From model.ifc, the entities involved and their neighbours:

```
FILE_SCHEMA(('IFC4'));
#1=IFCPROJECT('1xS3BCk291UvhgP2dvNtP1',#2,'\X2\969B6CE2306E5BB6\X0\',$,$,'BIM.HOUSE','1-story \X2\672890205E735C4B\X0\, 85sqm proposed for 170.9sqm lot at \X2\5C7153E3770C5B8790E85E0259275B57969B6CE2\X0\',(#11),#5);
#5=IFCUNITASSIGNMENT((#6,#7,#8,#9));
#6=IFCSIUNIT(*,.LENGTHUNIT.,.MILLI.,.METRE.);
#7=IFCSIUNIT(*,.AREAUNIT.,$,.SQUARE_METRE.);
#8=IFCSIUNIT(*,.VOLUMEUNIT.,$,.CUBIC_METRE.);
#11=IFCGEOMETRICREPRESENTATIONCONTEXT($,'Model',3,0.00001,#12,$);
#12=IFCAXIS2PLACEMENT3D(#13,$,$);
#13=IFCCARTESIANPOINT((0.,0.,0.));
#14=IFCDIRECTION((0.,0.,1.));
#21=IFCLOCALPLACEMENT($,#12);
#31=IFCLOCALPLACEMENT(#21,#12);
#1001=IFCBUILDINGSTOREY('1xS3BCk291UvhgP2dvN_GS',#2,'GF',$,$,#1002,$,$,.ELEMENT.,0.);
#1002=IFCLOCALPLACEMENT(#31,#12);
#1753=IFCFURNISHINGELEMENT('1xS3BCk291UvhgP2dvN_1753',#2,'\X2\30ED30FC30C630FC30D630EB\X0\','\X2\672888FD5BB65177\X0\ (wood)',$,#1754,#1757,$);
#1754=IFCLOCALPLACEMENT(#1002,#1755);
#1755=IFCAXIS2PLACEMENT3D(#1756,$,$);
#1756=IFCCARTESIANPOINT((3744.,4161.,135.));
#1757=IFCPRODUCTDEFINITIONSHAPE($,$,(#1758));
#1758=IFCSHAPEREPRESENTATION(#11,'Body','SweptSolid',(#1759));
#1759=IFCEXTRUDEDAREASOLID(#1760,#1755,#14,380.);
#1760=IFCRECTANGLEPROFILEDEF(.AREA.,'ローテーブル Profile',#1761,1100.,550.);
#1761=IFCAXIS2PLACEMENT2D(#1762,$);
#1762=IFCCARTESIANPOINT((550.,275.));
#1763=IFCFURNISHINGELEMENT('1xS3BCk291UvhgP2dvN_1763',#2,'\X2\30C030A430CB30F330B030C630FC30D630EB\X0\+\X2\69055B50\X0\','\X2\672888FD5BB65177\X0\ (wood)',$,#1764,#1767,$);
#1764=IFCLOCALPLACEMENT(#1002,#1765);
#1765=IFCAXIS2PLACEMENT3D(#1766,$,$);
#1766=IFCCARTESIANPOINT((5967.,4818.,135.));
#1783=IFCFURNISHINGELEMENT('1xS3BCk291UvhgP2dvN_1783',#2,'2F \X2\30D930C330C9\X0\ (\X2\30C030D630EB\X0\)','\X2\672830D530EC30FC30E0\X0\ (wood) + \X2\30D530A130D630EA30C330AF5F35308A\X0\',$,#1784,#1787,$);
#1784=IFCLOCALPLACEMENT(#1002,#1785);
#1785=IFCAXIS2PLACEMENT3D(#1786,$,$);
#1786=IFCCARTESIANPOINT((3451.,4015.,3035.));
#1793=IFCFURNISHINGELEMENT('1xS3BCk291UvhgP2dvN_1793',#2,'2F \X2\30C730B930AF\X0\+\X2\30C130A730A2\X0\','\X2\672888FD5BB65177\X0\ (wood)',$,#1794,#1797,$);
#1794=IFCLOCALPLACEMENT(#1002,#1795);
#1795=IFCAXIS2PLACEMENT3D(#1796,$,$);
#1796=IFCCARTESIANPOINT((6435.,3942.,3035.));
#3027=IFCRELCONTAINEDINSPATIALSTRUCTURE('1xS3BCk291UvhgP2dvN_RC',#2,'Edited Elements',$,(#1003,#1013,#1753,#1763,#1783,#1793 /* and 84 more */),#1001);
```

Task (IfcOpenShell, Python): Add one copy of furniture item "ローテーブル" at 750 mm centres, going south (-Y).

```python
import numpy as np
import ifcopenshell
import ifcopenshell.api.geometry
import ifcopenshell.api.root
import ifcopenshell.util.element
import ifcopenshell.util.placement
import ifcopenshell.util.unit

model = ifcopenshell.open("model.ifc")
unit_scale = ifcopenshell.util.unit.calculate_unit_scale(model)


def reuse_history(source, copy):
    """copy_class also copies each property set's owner history, people and application; keep the originals."""
    for rel in copy.IsDefinedBy:
        if rel.is_a("IfcRelDefinesByProperties") and (history := rel.RelatingPropertyDefinition.OwnerHistory):
            rel.RelatingPropertyDefinition.OwnerHistory = source.OwnerHistory
            ifcopenshell.util.element.remove_deep2(model, history)


source = model.by_guid("1xS3BCk291UvhgP2dvN_1753")
base = ifcopenshell.util.placement.get_local_placement(source.ObjectPlacement)
step = np.array([0.0, -1.0, 0.0]) * 0.75 / unit_scale

for i in range(1, 2):
    copy = ifcopenshell.api.root.copy_class(model, product=source)
    copy.Representation = ifcopenshell.util.element.copy_deep(
        model, source.Representation, exclude=["IfcGeometricRepresentationContext", "IfcRepresentationMap"]
    )
    reuse_history(source, copy)
    matrix = base.copy()
    matrix[:3, 3] += i * step
    print("added at", matrix[:3, 3].round(3) + 0.0)
    ifcopenshell.api.geometry.edit_object_placement(model, product=copy, matrix=matrix, is_si=False)

model.write("model_updated.ifc")
```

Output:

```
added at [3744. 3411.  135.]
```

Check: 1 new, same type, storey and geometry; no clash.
